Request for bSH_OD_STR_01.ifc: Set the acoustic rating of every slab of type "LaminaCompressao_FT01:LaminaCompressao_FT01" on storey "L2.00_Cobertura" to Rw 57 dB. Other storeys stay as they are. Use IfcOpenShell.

First a look at what the model holds.

```python
import ifcopenshell
import ifcopenshell.util.element

model = ifcopenshell.open("bSH_OD_STR_01.ifc")
print(model.schema)
storey = next(s for s in model.by_type("IfcBuildingStorey") if s.Name == "L2.00_Cobertura")
slabs = [e for e in ifcopenshell.util.element.get_decomposition(storey) if e.is_a("IfcSlab")]
seen = {}
for e in slabs:
    element_type = ifcopenshell.util.element.get_type(e)
    key = (element_type.Name if element_type != e and element_type else None, ifcopenshell.util.element.get_pset(e, "Pset_SlabCommon", "AcousticRating"))
    seen[key] = seen.get(key, 0) + 1
for (name, value), count in sorted(seen.items(), key=str):
    print(count, "x", name, "|", value)
```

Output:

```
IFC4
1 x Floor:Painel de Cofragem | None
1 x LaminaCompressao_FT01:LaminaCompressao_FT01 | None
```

```python
import ifcopenshell
import ifcopenshell.api.pset
import ifcopenshell.util.element

model = ifcopenshell.open("bSH_OD_STR_01.ifc")

storey = next(s for s in model.by_type("IfcBuildingStorey") if s.Name == "L2.00_Cobertura")
slabs = [e for e in ifcopenshell.util.element.get_decomposition(storey) if e.is_a("IfcSlab")]

count = 0
for e in slabs:
    element_type = ifcopenshell.util.element.get_type(e)
    if element_type in (None, e) or element_type.Name != "LaminaCompressao_FT01:LaminaCompressao_FT01":
        continue
    # add_pset returns the element's existing set when there is one.
    pset = ifcopenshell.api.pset.add_pset(model, product=e, name="Pset_SlabCommon")
    ifcopenshell.api.pset.edit_pset(model, pset=pset, properties={"AcousticRating": "Rw 57 dB"})
    count += 1

print(count, "slabs updated")

model.write("bSH_OD_STR_01_v2.ifc")
```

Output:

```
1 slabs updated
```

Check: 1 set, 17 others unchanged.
